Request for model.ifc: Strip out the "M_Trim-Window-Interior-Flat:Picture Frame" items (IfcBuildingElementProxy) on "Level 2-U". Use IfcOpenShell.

First a look at what the model holds.

```python
import ifcopenshell
import ifcopenshell.util.element

model = ifcopenshell.open("model.ifc")
print(model.schema)
storey = next(s for s in model.by_type("IfcBuildingStorey") if s.Name == "Level 2-U")
proxies = [e for e in ifcopenshell.util.element.get_decomposition(storey) if e.is_a("IfcBuildingElementProxy")]
seen = {}
for e in proxies:
    element_type = ifcopenshell.util.element.get_type(e)
    name = element_type.Name if element_type not in (None, e) else None
    seen[name] = seen.get(name, 0) + 1
for name, count in sorted(seen.items(), key=str):
    print(count, "x", name)
```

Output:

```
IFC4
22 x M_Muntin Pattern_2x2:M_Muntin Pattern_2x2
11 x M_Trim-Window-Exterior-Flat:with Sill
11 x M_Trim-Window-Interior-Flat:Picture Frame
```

```python
import ifcopenshell
import ifcopenshell.api.root
import ifcopenshell.util.element

model = ifcopenshell.open("model.ifc")

storey = next(s for s in model.by_type("IfcBuildingStorey") if s.Name == "Level 2-U")
proxies = [e for e in ifcopenshell.util.element.get_decomposition(storey) if e.is_a("IfcBuildingElementProxy")]
targets = [e for e in proxies if (t := ifcopenshell.util.element.get_type(e)) not in (None, e) and t.Name == "M_Trim-Window-Interior-Flat:Picture Frame"]

for e in targets:
    ifcopenshell.api.root.remove_product(model, product=e)
print(len(targets), "removed")

model.write("model_rev.ifc")
```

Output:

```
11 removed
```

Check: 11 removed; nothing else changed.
